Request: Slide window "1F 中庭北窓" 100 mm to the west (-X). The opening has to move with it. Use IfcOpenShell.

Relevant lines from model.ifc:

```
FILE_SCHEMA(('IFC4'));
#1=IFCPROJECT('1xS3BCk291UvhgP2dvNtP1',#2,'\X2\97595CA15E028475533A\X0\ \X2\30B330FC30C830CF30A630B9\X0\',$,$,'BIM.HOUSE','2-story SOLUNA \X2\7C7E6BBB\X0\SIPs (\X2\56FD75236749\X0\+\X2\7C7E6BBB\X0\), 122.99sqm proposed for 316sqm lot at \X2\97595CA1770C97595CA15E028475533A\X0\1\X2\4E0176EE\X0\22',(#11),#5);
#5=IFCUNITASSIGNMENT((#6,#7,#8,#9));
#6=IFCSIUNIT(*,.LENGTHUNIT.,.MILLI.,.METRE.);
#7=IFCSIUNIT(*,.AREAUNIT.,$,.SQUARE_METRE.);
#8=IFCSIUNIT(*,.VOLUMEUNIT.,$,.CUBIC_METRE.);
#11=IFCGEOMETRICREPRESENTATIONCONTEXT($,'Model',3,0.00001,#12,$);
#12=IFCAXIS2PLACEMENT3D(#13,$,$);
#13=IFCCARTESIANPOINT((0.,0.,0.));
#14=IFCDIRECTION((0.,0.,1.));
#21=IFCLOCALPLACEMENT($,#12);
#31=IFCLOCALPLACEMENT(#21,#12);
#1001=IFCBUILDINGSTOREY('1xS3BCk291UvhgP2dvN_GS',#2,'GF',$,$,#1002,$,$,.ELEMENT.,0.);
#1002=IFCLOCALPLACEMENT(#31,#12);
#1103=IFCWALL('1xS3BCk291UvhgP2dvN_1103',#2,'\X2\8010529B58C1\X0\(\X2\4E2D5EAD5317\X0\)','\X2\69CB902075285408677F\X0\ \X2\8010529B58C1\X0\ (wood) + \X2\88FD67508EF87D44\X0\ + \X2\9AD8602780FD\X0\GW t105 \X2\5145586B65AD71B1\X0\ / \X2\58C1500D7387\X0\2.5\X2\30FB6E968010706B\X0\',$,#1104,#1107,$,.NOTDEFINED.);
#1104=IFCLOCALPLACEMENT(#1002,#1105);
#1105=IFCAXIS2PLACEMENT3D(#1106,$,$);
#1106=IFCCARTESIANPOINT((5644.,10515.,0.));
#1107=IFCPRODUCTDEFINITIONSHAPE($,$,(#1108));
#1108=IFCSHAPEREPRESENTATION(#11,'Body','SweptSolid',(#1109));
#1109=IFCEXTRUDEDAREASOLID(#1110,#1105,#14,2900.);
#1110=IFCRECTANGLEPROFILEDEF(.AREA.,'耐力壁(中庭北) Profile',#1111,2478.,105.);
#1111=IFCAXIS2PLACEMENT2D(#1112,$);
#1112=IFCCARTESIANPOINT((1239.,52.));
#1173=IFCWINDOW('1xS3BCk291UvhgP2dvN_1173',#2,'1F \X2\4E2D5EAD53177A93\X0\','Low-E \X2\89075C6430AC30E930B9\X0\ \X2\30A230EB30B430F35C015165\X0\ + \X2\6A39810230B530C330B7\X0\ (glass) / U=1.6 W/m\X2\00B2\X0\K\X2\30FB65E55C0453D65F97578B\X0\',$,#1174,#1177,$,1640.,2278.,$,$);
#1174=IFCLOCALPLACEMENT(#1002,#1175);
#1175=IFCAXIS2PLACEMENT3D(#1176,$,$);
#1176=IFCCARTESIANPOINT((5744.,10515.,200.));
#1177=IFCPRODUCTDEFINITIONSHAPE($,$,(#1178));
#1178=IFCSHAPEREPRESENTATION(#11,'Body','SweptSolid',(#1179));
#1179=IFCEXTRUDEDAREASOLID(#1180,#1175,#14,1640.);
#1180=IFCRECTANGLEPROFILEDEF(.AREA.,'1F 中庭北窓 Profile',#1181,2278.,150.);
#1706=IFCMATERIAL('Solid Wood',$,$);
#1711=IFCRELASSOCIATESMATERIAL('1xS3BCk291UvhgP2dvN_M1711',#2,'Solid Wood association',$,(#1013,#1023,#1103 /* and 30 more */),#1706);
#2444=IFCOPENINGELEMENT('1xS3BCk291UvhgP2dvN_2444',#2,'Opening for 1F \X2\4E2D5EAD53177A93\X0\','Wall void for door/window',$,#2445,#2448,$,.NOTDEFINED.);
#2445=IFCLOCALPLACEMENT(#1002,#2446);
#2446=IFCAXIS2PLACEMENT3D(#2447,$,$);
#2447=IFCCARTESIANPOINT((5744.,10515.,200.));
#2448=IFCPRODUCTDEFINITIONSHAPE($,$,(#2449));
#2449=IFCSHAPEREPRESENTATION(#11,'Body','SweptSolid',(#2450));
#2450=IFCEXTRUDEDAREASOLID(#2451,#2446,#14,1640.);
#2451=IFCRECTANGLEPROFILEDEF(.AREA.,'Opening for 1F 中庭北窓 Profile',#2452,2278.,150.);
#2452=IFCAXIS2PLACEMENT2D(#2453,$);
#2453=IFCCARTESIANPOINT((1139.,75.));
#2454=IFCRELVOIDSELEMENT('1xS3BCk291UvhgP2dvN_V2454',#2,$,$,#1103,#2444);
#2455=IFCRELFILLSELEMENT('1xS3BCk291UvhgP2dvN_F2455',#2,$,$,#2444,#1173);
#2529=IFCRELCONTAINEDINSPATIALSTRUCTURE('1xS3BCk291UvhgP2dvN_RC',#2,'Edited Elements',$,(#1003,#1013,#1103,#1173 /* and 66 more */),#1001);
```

```python
import ifcopenshell
import ifcopenshell.api.geometry
import ifcopenshell.util.placement
import ifcopenshell.util.unit

model = ifcopenshell.open("model.ifc")
unit_scale = ifcopenshell.util.unit.calculate_unit_scale(model)

window = model.by_id(1173)
opening = window.FillsVoids[0].RelatingOpeningElement
wall = opening.VoidsElements[0].RelatingBuildingElement

wall_matrix = ifcopenshell.util.placement.get_local_placement(wall.ObjectPlacement)
shift = wall_matrix[:3, 0] * -0.1 / unit_scale
before = ifcopenshell.util.placement.get_local_placement(window.ObjectPlacement)[:3, 3].copy()

# The window is not placed relative to its opening, so move both.
for product in (opening, window):
    matrix = ifcopenshell.util.placement.get_local_placement(product.ObjectPlacement)
    matrix[:3, 3] += shift
    ifcopenshell.api.geometry.edit_object_placement(model, product=product, matrix=matrix, is_si=False)

after = ifcopenshell.util.placement.get_local_placement(window.ObjectPlacement)[:3, 3]
print("window moved by", (after - before).round(3) + 0.0)

model.write("model-out.ifc")
```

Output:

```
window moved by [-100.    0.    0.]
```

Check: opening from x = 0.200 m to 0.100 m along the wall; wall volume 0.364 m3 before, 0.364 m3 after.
